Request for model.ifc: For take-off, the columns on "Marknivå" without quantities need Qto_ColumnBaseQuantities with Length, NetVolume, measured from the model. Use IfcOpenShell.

First a look at what the model holds.

```python
import ifcopenshell
import ifcopenshell.util.element
import ifcopenshell.util.unit

model = ifcopenshell.open("model.ifc")
print(model.schema)
for unit_type in ("LENGTHUNIT", "AREAUNIT", "VOLUMEUNIT"):
    print(unit_type, ifcopenshell.util.unit.calculate_unit_scale(model, unit_type))
storey = next(s for s in model.by_type("IfcBuildingStorey") if s.Name == "Marknivå")
columns = [e for e in ifcopenshell.util.element.get_decomposition(storey) if e.is_a("IfcColumn")]
for e in sorted(columns, key=lambda e: e.id()):
    print(e.id(), e.is_a(), e.Name, list(ifcopenshell.util.element.get_psets(e, qtos_only=True)), sep=" | ")
```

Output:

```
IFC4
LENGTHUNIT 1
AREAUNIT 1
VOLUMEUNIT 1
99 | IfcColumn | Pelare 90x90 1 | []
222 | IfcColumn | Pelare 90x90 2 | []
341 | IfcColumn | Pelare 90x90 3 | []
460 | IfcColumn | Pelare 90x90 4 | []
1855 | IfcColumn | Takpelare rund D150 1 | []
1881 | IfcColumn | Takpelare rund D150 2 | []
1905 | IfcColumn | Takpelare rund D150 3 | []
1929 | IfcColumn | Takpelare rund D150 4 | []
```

```python
import ifcopenshell
import ifcopenshell.api.pset
import ifcopenshell.geom
import ifcopenshell.util.element
import ifcopenshell.util.shape
import ifcopenshell.util.unit

model = ifcopenshell.open("model.ifc")
unit_scale = ifcopenshell.util.unit.calculate_unit_scale(model)
volume_scale = ifcopenshell.util.unit.calculate_unit_scale(model, "VOLUMEUNIT")
settings = ifcopenshell.geom.settings()

storey = next(s for s in model.by_type("IfcBuildingStorey") if s.Name == "Marknivå")
columns = [e for e in ifcopenshell.util.element.get_decomposition(storey) if e.is_a("IfcColumn")]

for e in sorted(columns, key=lambda e: e.id()):
    if ifcopenshell.util.element.get_psets(e, qtos_only=True, should_inherit=False):
        continue
    # Geometry comes back in metres, in the element's own axes.
    shape = ifcopenshell.geom.create_shape(settings, e)
    values = {
        "Length": ifcopenshell.util.shape.get_z(shape.geometry) / unit_scale,
        "NetVolume": ifcopenshell.util.shape.get_volume(shape.geometry) / volume_scale,
    }
    qto = ifcopenshell.api.pset.add_qto(model, product=e, name="Qto_ColumnBaseQuantities")
    ifcopenshell.api.pset.edit_qto(model, qto=qto, properties=values)
    print(e.id(), {k: round(v, 3) for k, v in values.items()})

model.write("model-out.ifc")
```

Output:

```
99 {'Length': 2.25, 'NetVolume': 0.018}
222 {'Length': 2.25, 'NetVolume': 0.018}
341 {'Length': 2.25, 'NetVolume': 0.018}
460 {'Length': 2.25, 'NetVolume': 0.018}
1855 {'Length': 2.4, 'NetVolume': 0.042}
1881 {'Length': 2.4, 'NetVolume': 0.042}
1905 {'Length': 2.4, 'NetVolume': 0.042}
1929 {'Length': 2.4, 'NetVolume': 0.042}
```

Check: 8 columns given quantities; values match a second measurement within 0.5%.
